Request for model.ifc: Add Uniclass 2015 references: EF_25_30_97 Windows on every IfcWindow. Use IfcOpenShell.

First a look at what the model holds.

```python
import ifcopenshell

model = ifcopenshell.open("model.ifc")
print(model.schema)
print("classifications:", [c.Name for c in model.by_type("IfcClassification")])
for ifc_class in ("IfcDoor", "IfcRoof", "IfcStair", "IfcWall", "IfcWindow"):
    print(ifc_class, len(model.by_type(ifc_class)))
```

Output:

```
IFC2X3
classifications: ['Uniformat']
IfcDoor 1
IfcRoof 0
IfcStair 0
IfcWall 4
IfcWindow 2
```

```python
import ifcopenshell
import ifcopenshell.api.classification

model = ifcopenshell.open("model.ifc")

# IFC2X3 requires Source and Edition and has no link from the project to the system.
system = model.create_entity("IfcClassification", Source="NBS", Edition="2015", Name="Uniclass 2015")

codes = {
    "IfcWindow": ("EF_25_30_97", "Windows"),
}
for ifc_class, (code, name) in codes.items():
    products = model.by_type(ifc_class)
    ifcopenshell.api.classification.add_reference(
        model, products=products, classification=system, identification=code, name=name
    )
    print(code, len(products))

model.write("model_edited.ifc")
```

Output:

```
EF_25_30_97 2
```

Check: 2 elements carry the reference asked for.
